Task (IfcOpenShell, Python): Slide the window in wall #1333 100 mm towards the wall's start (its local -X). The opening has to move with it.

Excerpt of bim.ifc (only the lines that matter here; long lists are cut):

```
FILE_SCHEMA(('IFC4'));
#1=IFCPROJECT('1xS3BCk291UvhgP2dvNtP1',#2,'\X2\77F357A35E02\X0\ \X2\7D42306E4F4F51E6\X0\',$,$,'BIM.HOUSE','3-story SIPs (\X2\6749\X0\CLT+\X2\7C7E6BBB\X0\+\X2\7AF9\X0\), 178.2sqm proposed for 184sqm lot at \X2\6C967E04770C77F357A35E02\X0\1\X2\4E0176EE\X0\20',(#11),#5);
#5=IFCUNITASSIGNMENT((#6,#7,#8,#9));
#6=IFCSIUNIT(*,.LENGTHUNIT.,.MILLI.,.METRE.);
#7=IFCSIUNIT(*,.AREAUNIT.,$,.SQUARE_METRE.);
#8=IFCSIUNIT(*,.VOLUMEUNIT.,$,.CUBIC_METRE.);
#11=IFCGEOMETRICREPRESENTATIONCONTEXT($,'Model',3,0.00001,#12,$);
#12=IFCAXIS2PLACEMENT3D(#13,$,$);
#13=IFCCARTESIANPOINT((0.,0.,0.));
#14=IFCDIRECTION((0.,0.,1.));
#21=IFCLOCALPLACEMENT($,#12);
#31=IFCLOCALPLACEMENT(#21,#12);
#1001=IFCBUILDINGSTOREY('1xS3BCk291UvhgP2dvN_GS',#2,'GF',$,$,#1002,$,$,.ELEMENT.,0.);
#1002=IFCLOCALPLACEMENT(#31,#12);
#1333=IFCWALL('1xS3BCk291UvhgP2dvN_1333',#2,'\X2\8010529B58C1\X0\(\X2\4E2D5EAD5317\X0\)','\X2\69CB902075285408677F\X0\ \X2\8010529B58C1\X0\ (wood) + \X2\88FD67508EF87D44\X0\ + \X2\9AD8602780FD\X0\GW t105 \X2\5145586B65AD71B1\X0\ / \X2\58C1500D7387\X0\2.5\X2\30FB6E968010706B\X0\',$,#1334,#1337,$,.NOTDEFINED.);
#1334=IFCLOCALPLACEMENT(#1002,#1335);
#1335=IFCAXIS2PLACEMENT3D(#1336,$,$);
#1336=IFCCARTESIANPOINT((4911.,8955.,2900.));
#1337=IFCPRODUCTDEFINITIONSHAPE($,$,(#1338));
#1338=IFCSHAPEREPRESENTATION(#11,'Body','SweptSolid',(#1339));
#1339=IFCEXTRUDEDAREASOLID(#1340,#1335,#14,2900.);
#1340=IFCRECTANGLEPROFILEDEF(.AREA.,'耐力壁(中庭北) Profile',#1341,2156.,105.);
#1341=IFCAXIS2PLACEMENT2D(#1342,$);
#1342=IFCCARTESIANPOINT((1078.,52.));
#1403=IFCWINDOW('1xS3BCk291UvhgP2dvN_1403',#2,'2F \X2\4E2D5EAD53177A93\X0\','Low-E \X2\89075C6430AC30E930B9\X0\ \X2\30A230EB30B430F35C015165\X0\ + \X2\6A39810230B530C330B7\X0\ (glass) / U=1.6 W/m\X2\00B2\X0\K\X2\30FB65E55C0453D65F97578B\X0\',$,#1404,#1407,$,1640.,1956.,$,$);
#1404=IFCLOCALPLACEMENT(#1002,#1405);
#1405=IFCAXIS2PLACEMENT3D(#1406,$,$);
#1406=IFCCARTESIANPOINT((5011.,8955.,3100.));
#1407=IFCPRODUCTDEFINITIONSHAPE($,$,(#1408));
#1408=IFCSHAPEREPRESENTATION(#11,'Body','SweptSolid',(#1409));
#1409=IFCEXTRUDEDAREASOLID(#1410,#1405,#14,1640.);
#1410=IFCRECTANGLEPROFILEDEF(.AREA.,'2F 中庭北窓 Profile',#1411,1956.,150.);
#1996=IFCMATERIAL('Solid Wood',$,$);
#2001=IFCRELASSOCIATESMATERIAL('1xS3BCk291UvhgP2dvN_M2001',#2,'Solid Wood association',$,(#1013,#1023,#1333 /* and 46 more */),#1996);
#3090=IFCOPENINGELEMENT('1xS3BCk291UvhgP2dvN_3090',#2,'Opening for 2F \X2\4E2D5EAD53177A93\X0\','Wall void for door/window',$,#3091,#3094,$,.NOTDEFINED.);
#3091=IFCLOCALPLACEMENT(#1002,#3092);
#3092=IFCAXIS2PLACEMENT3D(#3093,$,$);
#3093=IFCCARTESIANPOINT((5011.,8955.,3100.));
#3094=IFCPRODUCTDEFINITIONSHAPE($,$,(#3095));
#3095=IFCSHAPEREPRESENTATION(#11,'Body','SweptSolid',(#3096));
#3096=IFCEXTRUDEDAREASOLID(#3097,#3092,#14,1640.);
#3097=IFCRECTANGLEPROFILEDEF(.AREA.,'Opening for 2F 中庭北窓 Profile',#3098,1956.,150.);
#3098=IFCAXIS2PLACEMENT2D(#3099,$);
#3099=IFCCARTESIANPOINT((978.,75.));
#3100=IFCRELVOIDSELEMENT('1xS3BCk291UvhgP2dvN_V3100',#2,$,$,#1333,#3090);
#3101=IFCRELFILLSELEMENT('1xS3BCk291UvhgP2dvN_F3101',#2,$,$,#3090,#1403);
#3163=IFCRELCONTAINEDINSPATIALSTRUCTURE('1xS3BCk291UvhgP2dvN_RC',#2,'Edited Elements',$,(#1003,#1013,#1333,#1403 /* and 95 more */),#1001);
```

```python
import ifcopenshell
import ifcopenshell.api.geometry
import ifcopenshell.util.placement
import ifcopenshell.util.unit

model = ifcopenshell.open("bim.ifc")
unit_scale = ifcopenshell.util.unit.calculate_unit_scale(model)

window = model.by_guid("1xS3BCk291UvhgP2dvN_1403")
opening = window.FillsVoids[0].RelatingOpeningElement
wall = opening.VoidsElements[0].RelatingBuildingElement

wall_matrix = ifcopenshell.util.placement.get_local_placement(wall.ObjectPlacement)
shift = wall_matrix[:3, 0] * -0.1 / unit_scale
before = ifcopenshell.util.placement.get_local_placement(window.ObjectPlacement)[:3, 3].copy()

# The window is not placed relative to its opening, so move both.
for product in (opening, window):
    matrix = ifcopenshell.util.placement.get_local_placement(product.ObjectPlacement)
    matrix[:3, 3] += shift
    ifcopenshell.api.geometry.edit_object_placement(model, product=product, matrix=matrix, is_si=False)

after = ifcopenshell.util.placement.get_local_placement(window.ObjectPlacement)[:3, 3]
print("window moved by", (after - before).round(3) + 0.0)

model.write("bim_updated.ifc")
```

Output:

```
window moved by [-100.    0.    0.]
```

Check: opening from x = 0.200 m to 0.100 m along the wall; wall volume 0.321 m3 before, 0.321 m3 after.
